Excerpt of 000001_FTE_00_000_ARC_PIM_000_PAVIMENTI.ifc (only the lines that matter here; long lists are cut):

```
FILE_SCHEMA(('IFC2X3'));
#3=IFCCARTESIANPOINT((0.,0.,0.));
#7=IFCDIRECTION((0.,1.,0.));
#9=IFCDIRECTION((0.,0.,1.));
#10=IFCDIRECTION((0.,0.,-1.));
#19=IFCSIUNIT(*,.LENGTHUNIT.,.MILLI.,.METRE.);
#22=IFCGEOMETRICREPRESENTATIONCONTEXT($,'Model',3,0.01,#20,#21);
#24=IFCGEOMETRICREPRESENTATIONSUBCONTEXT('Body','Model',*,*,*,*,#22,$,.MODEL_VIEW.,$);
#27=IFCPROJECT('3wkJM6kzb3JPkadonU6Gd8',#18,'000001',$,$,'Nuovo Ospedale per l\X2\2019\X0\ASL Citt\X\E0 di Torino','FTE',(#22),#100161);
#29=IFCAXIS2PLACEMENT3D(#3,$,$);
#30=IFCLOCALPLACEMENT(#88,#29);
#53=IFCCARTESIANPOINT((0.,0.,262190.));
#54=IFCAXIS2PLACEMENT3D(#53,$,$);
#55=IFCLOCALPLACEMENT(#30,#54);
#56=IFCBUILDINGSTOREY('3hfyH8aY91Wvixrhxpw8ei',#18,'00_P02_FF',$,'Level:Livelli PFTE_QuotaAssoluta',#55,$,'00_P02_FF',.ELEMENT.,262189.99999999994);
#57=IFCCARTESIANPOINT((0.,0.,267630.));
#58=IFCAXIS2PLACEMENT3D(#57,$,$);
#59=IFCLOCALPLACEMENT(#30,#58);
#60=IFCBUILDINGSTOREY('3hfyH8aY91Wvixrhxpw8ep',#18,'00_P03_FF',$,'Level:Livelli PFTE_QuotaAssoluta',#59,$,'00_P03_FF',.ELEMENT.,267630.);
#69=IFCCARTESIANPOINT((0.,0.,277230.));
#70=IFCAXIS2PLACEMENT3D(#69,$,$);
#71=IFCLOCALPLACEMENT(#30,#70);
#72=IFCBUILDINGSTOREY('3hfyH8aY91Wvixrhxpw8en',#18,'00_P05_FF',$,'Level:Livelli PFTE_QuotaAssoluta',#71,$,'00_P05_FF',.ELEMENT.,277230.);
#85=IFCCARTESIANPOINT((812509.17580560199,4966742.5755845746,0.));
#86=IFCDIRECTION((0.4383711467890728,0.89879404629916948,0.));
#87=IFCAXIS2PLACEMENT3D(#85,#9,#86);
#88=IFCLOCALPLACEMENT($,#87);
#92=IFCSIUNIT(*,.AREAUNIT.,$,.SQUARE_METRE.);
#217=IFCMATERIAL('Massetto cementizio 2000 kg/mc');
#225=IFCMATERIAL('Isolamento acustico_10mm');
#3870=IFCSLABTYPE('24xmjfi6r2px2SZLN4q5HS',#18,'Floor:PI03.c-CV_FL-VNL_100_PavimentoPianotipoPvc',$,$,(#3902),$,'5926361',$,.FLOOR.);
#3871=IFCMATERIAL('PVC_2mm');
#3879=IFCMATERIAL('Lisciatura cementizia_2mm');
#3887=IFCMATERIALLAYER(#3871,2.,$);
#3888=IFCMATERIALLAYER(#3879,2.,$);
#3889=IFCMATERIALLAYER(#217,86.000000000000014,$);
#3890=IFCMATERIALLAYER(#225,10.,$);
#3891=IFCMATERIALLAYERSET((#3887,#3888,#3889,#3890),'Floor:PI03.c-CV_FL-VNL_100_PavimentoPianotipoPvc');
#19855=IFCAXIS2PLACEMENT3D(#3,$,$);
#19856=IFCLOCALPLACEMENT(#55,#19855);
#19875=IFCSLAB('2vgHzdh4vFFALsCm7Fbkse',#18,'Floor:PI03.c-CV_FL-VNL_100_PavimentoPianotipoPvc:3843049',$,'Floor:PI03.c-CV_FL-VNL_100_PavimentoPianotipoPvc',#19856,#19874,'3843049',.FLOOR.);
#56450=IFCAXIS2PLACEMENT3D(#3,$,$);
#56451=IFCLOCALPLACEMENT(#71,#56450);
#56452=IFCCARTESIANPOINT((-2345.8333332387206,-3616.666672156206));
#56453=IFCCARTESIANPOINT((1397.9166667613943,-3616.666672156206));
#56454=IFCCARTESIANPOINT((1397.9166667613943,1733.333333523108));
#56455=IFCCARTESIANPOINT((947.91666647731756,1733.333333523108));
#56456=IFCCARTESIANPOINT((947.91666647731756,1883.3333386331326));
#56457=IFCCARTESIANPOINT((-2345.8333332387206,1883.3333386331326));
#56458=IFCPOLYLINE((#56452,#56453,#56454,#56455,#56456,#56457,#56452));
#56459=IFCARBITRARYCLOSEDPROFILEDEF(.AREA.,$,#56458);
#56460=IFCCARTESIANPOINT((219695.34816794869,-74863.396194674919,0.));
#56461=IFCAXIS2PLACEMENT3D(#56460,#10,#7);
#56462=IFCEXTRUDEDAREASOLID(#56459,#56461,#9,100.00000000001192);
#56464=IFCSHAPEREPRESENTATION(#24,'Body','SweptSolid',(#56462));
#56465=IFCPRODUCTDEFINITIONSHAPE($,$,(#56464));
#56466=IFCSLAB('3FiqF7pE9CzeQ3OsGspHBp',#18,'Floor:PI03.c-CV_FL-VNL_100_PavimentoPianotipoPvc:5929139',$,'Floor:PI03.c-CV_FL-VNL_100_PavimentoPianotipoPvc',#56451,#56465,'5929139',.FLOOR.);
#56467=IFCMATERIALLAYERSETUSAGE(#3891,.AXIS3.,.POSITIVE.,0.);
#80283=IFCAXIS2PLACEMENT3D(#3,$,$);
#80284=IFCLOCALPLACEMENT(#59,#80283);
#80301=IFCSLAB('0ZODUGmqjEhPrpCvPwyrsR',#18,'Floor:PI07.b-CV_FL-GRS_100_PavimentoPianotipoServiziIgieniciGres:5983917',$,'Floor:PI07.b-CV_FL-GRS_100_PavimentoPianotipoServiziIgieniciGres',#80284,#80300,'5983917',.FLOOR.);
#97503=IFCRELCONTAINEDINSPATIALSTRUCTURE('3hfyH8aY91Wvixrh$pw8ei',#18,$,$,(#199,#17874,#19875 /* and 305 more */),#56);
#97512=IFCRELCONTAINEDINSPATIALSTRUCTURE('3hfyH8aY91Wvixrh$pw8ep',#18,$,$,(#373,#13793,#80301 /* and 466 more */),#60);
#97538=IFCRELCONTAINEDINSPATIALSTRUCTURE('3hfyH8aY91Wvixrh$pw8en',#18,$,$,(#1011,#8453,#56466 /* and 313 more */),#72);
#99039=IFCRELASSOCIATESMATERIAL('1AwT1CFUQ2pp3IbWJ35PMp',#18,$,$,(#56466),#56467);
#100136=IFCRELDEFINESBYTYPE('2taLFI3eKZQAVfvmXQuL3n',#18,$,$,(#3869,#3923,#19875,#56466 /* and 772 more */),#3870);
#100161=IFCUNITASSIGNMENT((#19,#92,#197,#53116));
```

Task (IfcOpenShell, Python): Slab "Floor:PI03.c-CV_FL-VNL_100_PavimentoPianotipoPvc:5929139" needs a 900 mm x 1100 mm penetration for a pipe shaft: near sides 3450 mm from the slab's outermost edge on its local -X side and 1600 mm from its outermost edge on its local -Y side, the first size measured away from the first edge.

```python
import numpy as np
import ifcopenshell
import ifcopenshell.api.feature
import ifcopenshell.api.geometry
import ifcopenshell.api.root
import ifcopenshell.geom
import ifcopenshell.util.placement
import ifcopenshell.util.representation
import ifcopenshell.util.shape
import ifcopenshell.util.unit

model = ifcopenshell.open("000001_FTE_00_000_ARC_PIM_000_PAVIMENTI.ifc")
unit_scale = ifcopenshell.util.unit.calculate_unit_scale(model)
settings = ifcopenshell.geom.settings()


def volume(element):
    """Net volume in cubic metres, openings subtracted."""
    shape = ifcopenshell.geom.create_shape(settings, element)
    return ifcopenshell.util.shape.get_volume(shape.geometry)


slab = model.by_guid("3FiqF7pE9CzeQ3OsGspHBp")
before = volume(slab)

# Extent in the slab's own axes, in metres. The edges named are its -X and -Y sides.
slab_shape = ifcopenshell.geom.create_shape(settings, slab)
vertices = ifcopenshell.util.shape.get_vertices(slab_shape.geometry)
x_min, y_min, bottom = vertices.min(axis=0)
top = vertices[:, 2].max()

opening = ifcopenshell.api.root.create_entity(model, ifc_class="IfcOpeningElement", name="Pipe shaft opening")
context = ifcopenshell.util.representation.get_context(model, "Model", "Body", "MODEL_VIEW")
width, depth = 0.9, 1.1
outline = [(0.0, 0.0), (width, 0.0), (width, depth), (0.0, depth), (0.0, 0.0)]
# Overshoot both faces by 50 mm so the cut is clean.
shape = ifcopenshell.api.geometry.add_slab_representation(
    model, context=context, depth=top - bottom + 0.1, polyline=outline
)
ifcopenshell.api.geometry.assign_representation(model, product=opening, representation=shape)

matrix = ifcopenshell.util.placement.get_local_placement(slab.ObjectPlacement)
matrix[:, 3] = matrix @ np.append(np.array([x_min + 3.45, y_min + 1.6, bottom - 0.05]) / unit_scale, 1.0)
ifcopenshell.api.geometry.edit_object_placement(model, product=opening, matrix=matrix, is_si=False)
ifcopenshell.api.feature.add_feature(model, feature=opening, element=slab)

after = volume(slab)

print(f"slab volume {before:.3f} -> {after:.3f} m3")

model.write("000001_FTE_00_000_ARC_PIM_000_PAVIMENTI_updated.ifc")
```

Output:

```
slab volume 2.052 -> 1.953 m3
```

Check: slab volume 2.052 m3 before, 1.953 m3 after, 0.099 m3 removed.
